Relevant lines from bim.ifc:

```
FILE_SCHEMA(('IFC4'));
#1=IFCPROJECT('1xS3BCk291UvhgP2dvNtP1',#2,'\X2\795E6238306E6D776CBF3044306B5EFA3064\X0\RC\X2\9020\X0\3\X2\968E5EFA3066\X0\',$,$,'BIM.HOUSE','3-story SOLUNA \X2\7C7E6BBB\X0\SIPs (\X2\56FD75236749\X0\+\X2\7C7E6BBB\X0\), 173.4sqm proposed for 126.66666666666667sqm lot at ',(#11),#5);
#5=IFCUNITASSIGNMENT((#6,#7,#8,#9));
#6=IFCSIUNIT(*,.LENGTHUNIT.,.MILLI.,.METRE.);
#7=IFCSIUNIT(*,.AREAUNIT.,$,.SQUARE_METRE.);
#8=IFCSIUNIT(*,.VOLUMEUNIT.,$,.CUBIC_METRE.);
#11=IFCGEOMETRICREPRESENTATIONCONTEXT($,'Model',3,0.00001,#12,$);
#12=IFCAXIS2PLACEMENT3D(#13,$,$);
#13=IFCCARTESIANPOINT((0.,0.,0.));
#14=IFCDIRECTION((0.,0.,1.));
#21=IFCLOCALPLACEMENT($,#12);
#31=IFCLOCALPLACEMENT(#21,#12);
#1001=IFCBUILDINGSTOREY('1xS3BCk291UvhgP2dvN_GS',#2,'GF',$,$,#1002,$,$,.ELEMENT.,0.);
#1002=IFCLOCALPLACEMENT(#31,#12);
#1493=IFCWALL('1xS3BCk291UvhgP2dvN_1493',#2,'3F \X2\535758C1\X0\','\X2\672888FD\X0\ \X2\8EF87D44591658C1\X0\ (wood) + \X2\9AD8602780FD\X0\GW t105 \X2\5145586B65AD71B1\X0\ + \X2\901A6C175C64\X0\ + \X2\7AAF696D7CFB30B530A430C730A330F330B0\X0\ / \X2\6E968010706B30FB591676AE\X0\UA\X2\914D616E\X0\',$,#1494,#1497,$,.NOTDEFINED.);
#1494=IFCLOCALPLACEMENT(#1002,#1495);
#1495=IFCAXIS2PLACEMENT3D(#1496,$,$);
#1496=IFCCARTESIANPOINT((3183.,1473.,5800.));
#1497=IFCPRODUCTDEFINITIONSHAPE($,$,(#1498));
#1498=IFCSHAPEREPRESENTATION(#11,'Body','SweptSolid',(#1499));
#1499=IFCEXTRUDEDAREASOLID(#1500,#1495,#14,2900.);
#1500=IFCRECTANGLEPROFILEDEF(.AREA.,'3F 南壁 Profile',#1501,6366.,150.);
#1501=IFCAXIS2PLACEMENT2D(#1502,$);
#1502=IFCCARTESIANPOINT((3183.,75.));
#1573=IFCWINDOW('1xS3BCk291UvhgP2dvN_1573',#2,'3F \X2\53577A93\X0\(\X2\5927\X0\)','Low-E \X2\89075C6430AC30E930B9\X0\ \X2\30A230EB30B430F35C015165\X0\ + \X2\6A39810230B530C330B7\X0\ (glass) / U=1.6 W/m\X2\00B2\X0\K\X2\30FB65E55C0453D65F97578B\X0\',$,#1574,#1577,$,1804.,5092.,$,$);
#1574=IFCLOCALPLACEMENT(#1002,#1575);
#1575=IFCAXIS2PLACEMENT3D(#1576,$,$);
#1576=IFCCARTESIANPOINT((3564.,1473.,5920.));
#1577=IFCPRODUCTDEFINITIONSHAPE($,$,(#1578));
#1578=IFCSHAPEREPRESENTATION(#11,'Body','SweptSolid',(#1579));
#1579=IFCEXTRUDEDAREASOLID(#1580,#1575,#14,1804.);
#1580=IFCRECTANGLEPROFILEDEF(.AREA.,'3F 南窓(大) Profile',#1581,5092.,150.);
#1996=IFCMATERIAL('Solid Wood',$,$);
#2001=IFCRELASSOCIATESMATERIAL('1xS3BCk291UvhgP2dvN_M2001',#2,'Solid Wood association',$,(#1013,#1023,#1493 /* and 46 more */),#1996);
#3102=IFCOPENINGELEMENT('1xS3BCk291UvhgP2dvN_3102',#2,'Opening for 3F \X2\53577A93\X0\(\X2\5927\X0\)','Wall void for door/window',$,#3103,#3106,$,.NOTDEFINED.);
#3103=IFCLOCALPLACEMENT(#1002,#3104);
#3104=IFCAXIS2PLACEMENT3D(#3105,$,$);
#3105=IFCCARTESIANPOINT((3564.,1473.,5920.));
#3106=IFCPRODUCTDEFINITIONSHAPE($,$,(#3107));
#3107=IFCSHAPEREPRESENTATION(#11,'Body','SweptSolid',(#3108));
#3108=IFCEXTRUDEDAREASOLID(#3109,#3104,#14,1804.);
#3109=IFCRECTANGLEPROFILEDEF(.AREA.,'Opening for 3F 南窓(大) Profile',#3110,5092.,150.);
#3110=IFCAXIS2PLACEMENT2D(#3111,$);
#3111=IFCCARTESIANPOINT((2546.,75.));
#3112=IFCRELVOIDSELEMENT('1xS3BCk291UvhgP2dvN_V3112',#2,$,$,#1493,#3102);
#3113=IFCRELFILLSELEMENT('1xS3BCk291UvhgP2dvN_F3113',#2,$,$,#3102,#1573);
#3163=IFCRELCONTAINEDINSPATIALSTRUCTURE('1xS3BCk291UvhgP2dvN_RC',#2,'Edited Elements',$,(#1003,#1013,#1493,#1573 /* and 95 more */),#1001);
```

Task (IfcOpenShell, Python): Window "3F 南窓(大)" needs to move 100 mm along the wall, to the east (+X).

```python
import ifcopenshell
import ifcopenshell.api.geometry
import ifcopenshell.util.placement

model = ifcopenshell.open("bim.ifc")

window = model.by_id(1573)
opening = window.FillsVoids[0].RelatingOpeningElement
wall = opening.VoidsElements[0].RelatingBuildingElement

wall_matrix = ifcopenshell.util.placement.get_local_placement(wall.ObjectPlacement)
shift = wall_matrix[:3, 0] * 100.0
before = ifcopenshell.util.placement.get_local_placement(window.ObjectPlacement)[:3, 3].copy()

# The window is not placed relative to its opening, so move both.
for product in (opening, window):
    matrix = ifcopenshell.util.placement.get_local_placement(product.ObjectPlacement)
    matrix[:3, 3] += shift
    ifcopenshell.api.geometry.edit_object_placement(model, product=product, matrix=matrix, is_si=False)

after = ifcopenshell.util.placement.get_local_placement(window.ObjectPlacement)[:3, 3]
print("window moved by", (after - before).round(3) + 0.0)

model.write("bim_v2.ifc")
```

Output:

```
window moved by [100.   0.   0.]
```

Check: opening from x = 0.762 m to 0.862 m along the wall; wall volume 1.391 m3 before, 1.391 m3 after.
